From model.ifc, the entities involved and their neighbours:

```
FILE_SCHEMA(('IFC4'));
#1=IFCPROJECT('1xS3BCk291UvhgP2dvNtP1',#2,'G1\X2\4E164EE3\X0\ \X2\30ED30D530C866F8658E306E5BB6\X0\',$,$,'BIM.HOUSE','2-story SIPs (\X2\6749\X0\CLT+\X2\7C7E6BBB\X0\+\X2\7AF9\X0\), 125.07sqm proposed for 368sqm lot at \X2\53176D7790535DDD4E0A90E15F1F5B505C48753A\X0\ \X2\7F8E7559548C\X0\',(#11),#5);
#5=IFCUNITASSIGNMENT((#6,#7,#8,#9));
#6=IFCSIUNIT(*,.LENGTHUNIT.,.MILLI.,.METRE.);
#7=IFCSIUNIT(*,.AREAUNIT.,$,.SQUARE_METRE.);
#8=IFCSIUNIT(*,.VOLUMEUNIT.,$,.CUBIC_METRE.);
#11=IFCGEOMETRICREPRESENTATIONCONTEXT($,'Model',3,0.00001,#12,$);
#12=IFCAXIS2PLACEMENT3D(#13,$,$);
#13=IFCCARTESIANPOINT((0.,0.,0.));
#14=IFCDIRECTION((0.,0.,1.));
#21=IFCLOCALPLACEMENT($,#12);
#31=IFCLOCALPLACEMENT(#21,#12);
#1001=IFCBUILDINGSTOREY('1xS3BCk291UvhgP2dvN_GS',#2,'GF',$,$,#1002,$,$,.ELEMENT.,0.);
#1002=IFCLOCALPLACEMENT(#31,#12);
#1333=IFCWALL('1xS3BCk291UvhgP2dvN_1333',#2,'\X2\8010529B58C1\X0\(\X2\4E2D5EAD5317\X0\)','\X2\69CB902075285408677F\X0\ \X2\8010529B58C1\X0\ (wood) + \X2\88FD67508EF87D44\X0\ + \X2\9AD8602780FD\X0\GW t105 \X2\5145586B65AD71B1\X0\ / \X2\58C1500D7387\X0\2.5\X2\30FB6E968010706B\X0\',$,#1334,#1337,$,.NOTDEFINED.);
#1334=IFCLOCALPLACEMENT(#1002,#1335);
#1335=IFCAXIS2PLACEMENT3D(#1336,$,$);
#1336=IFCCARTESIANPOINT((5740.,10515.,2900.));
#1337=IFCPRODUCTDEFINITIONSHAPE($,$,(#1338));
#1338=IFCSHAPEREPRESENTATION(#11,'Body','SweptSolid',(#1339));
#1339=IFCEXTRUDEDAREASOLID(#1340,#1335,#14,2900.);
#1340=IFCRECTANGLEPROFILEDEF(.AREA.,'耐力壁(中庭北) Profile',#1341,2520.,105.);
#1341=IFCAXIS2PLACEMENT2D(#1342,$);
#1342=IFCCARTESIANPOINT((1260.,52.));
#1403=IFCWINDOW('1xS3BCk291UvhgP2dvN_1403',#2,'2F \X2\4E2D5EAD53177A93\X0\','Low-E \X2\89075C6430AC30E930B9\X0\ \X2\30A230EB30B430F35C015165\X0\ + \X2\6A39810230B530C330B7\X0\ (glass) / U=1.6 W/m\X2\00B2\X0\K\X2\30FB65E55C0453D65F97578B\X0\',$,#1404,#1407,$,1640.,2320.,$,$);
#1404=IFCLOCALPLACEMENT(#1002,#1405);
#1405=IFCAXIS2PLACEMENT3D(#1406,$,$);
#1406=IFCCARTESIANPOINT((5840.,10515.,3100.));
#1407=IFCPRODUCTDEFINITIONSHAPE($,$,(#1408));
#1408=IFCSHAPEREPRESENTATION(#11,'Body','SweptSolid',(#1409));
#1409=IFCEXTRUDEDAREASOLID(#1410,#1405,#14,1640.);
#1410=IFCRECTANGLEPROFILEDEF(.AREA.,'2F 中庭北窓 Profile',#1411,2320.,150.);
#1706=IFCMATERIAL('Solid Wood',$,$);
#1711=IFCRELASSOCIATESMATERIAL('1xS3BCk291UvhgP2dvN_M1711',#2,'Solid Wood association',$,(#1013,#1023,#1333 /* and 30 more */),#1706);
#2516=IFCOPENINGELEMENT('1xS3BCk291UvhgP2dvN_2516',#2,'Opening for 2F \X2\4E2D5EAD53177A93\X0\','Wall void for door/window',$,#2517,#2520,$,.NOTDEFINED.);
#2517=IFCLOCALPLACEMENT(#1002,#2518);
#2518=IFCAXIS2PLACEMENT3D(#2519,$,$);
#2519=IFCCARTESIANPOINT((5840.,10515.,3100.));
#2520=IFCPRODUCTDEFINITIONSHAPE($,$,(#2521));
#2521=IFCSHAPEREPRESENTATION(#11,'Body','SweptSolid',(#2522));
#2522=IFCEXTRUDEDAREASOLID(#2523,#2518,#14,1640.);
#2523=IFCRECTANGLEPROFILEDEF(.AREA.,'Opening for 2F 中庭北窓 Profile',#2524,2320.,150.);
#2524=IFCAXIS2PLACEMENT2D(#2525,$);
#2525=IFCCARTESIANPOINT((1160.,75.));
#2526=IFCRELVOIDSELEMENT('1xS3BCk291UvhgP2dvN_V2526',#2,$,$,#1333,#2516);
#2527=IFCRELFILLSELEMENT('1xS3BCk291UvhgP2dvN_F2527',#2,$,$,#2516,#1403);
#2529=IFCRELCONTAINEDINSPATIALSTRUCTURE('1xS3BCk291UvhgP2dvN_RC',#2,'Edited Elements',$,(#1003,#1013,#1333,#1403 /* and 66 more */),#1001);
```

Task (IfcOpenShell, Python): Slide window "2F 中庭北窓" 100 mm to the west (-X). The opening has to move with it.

```python
import ifcopenshell
import ifcopenshell.api.geometry
import ifcopenshell.util.placement

model = ifcopenshell.open("model.ifc")

window = model.by_id(1403)
opening = window.FillsVoids[0].RelatingOpeningElement
wall = opening.VoidsElements[0].RelatingBuildingElement

wall_matrix = ifcopenshell.util.placement.get_local_placement(wall.ObjectPlacement)
shift = wall_matrix[:3, 0] * -100.0
before = ifcopenshell.util.placement.get_local_placement(window.ObjectPlacement)[:3, 3].copy()

# The window is not placed relative to its opening, so move both.
for product in (opening, window):
    matrix = ifcopenshell.util.placement.get_local_placement(product.ObjectPlacement)
    matrix[:3, 3] += shift
    ifcopenshell.api.geometry.edit_object_placement(model, product=product, matrix=matrix, is_si=False)

after = ifcopenshell.util.placement.get_local_placement(window.ObjectPlacement)[:3, 3]
print("window moved by", (after - before).round(3) + 0.0)

model.write("model_updated.ifc")
```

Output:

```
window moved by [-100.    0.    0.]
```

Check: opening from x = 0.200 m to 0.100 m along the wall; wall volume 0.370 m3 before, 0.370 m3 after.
